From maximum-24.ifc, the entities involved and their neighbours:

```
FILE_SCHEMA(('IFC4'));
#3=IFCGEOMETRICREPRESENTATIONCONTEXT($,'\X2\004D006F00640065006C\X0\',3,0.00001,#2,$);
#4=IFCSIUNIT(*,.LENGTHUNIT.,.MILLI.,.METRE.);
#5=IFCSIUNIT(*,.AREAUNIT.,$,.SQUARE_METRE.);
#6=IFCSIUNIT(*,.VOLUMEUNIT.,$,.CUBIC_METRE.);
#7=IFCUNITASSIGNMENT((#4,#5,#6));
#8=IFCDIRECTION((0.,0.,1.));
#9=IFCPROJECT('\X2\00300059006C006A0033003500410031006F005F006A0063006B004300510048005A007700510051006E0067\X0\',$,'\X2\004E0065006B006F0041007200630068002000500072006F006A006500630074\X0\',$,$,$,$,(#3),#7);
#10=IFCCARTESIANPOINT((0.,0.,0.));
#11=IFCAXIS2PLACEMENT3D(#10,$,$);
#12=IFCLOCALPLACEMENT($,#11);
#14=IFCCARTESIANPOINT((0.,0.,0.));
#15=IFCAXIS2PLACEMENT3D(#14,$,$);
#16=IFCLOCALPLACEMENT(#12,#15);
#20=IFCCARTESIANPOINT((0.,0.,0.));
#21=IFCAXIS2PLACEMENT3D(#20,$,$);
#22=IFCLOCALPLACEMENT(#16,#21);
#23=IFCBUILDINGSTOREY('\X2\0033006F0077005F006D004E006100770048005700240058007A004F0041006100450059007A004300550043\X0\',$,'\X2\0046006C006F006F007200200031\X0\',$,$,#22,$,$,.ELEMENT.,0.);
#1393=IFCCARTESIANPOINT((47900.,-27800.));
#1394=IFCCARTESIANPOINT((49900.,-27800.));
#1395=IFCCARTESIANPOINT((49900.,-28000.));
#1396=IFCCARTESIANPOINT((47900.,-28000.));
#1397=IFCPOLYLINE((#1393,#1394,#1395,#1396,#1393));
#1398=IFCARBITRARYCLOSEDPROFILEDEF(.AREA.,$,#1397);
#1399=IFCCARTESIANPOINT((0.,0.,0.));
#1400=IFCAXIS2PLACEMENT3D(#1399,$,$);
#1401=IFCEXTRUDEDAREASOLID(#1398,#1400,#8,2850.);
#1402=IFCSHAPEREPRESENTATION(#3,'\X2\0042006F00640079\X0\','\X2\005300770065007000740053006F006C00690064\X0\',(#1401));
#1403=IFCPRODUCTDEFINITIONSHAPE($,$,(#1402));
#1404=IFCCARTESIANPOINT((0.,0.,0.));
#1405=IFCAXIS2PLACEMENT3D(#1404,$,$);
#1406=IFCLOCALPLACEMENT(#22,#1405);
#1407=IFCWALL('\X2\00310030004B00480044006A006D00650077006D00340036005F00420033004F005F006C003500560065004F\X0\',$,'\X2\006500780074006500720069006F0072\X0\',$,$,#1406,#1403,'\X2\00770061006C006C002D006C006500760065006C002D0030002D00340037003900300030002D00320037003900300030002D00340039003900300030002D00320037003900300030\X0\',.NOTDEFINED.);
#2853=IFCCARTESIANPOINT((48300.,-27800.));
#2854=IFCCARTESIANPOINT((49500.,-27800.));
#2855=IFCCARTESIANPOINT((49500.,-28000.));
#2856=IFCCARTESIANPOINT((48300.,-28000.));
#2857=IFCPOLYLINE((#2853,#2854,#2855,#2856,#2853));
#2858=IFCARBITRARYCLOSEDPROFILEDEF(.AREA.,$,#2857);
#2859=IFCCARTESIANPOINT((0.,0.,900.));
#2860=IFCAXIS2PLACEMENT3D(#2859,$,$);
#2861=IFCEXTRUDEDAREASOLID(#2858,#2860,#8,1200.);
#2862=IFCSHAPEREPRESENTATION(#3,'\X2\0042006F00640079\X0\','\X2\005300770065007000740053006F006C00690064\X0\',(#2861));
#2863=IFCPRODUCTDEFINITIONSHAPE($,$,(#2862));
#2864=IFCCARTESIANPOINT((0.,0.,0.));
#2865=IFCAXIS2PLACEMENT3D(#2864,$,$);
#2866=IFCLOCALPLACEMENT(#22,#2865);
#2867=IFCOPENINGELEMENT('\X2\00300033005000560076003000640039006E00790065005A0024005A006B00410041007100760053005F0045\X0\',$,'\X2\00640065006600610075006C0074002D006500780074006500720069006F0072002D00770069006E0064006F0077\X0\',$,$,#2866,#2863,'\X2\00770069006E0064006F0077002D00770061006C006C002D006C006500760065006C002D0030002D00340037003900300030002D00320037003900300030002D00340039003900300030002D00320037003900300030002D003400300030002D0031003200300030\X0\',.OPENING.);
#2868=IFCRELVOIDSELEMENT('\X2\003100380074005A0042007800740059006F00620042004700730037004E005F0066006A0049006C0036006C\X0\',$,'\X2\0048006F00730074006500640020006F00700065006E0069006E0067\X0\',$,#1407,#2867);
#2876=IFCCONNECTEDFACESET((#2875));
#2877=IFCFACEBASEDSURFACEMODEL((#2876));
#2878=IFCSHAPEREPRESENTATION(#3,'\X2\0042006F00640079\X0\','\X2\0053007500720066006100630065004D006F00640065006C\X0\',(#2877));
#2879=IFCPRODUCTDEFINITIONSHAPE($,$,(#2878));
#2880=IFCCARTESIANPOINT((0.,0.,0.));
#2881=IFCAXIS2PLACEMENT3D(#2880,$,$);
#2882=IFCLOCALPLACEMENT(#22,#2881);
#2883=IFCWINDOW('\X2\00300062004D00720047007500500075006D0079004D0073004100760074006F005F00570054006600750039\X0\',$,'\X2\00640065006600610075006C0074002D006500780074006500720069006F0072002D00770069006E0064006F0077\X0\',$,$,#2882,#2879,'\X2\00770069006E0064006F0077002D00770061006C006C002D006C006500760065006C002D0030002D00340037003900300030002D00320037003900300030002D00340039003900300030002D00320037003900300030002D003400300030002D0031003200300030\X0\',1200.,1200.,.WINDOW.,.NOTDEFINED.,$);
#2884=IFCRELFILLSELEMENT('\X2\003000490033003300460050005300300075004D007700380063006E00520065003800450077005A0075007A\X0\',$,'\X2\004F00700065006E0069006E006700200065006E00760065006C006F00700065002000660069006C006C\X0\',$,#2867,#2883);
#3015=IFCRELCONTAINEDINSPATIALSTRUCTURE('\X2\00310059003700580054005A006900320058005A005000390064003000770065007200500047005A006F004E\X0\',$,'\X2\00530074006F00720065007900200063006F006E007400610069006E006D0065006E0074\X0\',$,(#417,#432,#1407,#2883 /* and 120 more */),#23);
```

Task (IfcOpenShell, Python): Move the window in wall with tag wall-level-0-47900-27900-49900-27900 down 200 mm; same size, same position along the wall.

```python
import numpy as np
import ifcopenshell
import ifcopenshell.api.geometry
import ifcopenshell.util.placement
import ifcopenshell.util.unit

model = ifcopenshell.open("maximum-24.ifc")
unit_scale = ifcopenshell.util.unit.calculate_unit_scale(model)

window = model.by_id(2883)
opening = window.FillsVoids[0].RelatingOpeningElement
dz = -0.2 / unit_scale

shift = np.array([0.0, 0.0, dz])
# The window is not placed relative to its opening, so move both.
for product in (opening, window):
    matrix = ifcopenshell.util.placement.get_local_placement(product.ObjectPlacement)
    matrix[:3, 3] += shift
    ifcopenshell.api.geometry.edit_object_placement(model, product=product, matrix=matrix, is_si=False)

print(f"moved by {dz * unit_scale:+.3f} m")

model.write("maximum-24-out.ifc")
```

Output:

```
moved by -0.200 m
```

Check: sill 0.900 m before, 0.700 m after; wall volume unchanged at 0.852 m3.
